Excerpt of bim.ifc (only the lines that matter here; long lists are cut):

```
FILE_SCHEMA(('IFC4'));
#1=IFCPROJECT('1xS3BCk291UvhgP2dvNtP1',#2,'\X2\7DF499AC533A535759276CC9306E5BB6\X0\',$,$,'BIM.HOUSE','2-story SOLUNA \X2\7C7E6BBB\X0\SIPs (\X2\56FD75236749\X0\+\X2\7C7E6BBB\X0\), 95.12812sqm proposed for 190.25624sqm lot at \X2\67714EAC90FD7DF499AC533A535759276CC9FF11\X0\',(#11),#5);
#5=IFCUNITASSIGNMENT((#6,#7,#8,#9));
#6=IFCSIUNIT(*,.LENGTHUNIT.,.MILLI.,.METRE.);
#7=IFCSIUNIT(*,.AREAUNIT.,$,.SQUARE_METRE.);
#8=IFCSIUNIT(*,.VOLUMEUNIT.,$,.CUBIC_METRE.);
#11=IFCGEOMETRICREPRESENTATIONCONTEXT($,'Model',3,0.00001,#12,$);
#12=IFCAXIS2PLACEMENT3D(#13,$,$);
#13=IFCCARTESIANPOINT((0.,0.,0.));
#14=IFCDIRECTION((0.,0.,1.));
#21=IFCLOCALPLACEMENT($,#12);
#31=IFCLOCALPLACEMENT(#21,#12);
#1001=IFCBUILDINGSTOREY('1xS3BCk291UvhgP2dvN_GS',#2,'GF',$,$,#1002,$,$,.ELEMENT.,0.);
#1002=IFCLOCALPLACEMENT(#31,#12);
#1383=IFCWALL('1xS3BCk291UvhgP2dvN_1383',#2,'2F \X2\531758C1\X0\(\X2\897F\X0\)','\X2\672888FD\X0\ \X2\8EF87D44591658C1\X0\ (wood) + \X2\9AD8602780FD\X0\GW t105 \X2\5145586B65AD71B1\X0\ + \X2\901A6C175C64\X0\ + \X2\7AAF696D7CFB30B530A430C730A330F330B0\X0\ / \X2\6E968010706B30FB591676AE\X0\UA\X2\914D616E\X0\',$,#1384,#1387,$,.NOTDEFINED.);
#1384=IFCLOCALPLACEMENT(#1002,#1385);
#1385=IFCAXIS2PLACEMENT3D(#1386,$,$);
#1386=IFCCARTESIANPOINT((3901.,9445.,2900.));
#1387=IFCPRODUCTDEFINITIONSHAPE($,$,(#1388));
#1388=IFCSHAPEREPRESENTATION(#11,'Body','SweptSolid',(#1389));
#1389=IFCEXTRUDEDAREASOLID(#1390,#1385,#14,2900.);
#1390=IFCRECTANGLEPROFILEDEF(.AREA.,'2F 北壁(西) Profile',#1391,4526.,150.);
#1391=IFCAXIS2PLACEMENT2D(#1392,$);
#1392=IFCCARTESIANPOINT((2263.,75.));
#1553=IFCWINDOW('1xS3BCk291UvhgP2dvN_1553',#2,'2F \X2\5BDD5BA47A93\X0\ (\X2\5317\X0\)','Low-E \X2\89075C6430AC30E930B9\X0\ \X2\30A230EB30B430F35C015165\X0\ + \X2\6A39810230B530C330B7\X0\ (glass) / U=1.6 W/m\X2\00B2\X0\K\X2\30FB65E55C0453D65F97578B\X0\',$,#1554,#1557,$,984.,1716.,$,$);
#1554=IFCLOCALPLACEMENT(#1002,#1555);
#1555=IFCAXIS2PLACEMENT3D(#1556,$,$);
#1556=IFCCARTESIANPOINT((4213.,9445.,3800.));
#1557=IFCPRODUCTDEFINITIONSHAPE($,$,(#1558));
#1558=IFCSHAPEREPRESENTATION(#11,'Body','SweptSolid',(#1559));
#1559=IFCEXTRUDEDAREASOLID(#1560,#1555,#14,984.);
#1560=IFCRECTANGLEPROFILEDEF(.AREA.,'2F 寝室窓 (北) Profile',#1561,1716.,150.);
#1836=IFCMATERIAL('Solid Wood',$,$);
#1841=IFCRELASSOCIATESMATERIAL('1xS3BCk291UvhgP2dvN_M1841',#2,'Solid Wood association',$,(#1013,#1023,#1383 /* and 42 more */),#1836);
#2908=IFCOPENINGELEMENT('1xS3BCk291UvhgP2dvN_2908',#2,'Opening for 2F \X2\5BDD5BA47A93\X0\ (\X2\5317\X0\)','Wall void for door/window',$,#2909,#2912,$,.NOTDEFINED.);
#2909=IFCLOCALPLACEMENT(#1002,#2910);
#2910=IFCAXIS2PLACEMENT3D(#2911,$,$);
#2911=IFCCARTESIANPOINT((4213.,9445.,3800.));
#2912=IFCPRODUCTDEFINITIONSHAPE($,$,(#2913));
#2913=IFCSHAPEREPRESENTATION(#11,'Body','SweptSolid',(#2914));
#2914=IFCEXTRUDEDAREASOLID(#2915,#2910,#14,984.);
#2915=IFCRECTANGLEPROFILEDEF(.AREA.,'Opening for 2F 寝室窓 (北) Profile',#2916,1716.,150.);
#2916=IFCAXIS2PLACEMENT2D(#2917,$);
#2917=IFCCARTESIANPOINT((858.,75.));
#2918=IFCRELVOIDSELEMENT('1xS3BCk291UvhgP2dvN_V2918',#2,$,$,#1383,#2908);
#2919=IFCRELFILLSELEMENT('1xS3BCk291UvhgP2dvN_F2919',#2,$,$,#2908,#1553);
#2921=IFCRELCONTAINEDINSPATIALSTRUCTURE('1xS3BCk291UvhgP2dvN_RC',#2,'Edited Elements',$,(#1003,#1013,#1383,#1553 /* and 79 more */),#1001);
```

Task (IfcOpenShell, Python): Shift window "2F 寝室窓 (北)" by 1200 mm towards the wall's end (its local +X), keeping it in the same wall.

```python
import ifcopenshell
import ifcopenshell.api.geometry
import ifcopenshell.util.placement

model = ifcopenshell.open("bim.ifc")

window = model.by_id(1553)
opening = window.FillsVoids[0].RelatingOpeningElement
wall = opening.VoidsElements[0].RelatingBuildingElement

wall_matrix = ifcopenshell.util.placement.get_local_placement(wall.ObjectPlacement)
shift = wall_matrix[:3, 0] * 1200.0
before = ifcopenshell.util.placement.get_local_placement(window.ObjectPlacement)[:3, 3].copy()

# The window is not placed relative to its opening, so move both.
for product in (opening, window):
    matrix = ifcopenshell.util.placement.get_local_placement(product.ObjectPlacement)
    matrix[:3, 3] += shift
    ifcopenshell.api.geometry.edit_object_placement(model, product=product, matrix=matrix, is_si=False)

after = ifcopenshell.util.placement.get_local_placement(window.ObjectPlacement)[:3, 3]
print("window moved by", (after - before).round(3) + 0.0)

model.write("bim_edited.ifc")
```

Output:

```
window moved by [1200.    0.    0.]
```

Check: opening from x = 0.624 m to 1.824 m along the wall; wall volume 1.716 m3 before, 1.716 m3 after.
